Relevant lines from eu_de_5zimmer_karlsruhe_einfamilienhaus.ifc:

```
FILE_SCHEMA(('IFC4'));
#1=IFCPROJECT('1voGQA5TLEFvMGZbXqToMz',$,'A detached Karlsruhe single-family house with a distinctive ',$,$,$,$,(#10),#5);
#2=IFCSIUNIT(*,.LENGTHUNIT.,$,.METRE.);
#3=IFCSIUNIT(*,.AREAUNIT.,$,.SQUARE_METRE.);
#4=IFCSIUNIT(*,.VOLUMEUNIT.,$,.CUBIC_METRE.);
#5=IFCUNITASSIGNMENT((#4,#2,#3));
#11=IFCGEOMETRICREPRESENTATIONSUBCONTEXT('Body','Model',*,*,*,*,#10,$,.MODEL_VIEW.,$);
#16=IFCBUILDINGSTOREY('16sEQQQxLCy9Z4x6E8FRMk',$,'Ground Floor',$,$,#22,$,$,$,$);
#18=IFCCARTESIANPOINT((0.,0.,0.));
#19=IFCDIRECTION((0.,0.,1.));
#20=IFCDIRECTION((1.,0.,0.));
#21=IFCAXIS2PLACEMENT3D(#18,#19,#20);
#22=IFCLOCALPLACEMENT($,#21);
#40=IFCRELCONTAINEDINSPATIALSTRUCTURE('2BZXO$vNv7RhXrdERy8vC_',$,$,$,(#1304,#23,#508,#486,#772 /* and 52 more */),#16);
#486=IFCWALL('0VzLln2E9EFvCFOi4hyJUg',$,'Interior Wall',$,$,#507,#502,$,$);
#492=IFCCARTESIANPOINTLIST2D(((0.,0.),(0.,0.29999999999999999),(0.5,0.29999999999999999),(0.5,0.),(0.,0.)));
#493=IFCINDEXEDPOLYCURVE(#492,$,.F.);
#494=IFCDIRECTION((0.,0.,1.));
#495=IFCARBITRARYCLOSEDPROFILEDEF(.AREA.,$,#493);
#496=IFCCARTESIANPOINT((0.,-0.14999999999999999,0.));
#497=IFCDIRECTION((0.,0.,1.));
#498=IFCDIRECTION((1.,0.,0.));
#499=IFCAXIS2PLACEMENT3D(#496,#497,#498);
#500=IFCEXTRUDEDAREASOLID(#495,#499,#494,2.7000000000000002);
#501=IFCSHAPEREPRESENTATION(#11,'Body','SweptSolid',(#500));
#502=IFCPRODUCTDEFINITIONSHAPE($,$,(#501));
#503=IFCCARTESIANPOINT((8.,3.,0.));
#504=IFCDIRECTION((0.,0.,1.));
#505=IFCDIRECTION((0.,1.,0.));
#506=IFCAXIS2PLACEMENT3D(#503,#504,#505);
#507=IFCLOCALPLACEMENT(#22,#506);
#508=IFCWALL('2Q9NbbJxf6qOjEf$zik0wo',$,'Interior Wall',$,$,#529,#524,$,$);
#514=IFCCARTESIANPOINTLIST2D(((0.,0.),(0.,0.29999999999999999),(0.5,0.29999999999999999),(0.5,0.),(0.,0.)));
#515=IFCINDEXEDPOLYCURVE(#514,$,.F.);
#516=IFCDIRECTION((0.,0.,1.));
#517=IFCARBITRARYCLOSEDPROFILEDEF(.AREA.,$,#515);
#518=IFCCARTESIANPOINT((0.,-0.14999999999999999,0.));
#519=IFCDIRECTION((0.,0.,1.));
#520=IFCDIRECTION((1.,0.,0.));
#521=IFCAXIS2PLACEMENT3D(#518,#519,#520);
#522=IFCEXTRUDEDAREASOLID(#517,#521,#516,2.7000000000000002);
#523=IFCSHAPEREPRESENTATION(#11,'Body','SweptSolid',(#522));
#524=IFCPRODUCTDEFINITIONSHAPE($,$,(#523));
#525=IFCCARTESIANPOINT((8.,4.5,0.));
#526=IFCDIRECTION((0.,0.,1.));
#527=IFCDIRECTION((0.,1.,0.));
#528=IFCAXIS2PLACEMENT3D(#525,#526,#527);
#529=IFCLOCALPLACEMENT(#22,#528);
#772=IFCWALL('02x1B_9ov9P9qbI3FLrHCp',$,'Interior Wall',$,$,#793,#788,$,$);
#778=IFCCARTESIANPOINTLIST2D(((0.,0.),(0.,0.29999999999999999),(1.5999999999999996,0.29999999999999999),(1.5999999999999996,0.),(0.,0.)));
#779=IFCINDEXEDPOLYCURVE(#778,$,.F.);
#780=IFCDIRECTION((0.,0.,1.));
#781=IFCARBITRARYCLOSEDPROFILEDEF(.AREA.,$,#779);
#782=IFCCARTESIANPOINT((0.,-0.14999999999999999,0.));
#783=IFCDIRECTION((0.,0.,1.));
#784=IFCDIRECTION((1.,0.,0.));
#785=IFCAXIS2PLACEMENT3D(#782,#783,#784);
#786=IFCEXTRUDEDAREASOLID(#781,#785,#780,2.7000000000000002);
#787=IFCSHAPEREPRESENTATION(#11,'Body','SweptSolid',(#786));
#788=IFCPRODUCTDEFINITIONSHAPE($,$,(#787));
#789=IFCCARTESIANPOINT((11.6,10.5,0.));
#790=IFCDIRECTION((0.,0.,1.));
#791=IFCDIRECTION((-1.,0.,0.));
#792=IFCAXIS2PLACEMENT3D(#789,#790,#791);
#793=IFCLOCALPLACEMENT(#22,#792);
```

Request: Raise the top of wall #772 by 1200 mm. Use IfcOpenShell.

```python
import ifcopenshell
import ifcopenshell.geom
import ifcopenshell.util.representation
import ifcopenshell.util.shape

model = ifcopenshell.open("eu_de_5zimmer_karlsruhe_einfamilienhaus.ifc")
settings = ifcopenshell.geom.settings()


def volume(element):
    """Net volume in cubic metres, openings subtracted."""
    shape = ifcopenshell.geom.create_shape(settings, element)
    return ifcopenshell.util.shape.get_volume(shape.geometry)


wall = model.by_guid("02x1B_9ov9P9qbI3FLrHCp")
before = volume(wall)

body = ifcopenshell.util.representation.get_representation(wall, "Model", "Body")
solid = body.Items[0]
old_height = solid.Depth
solid.Depth += 1.2
after = volume(wall)

print(f"height {old_height:g} -> {solid.Depth:g}, volume {before:.3f} -> {after:.3f} m3")

model.write("eu_de_5zimmer_karlsruhe_einfamilienhaus-out.ifc")
```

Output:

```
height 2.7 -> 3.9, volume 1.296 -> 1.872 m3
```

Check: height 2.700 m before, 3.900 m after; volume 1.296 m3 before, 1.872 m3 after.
